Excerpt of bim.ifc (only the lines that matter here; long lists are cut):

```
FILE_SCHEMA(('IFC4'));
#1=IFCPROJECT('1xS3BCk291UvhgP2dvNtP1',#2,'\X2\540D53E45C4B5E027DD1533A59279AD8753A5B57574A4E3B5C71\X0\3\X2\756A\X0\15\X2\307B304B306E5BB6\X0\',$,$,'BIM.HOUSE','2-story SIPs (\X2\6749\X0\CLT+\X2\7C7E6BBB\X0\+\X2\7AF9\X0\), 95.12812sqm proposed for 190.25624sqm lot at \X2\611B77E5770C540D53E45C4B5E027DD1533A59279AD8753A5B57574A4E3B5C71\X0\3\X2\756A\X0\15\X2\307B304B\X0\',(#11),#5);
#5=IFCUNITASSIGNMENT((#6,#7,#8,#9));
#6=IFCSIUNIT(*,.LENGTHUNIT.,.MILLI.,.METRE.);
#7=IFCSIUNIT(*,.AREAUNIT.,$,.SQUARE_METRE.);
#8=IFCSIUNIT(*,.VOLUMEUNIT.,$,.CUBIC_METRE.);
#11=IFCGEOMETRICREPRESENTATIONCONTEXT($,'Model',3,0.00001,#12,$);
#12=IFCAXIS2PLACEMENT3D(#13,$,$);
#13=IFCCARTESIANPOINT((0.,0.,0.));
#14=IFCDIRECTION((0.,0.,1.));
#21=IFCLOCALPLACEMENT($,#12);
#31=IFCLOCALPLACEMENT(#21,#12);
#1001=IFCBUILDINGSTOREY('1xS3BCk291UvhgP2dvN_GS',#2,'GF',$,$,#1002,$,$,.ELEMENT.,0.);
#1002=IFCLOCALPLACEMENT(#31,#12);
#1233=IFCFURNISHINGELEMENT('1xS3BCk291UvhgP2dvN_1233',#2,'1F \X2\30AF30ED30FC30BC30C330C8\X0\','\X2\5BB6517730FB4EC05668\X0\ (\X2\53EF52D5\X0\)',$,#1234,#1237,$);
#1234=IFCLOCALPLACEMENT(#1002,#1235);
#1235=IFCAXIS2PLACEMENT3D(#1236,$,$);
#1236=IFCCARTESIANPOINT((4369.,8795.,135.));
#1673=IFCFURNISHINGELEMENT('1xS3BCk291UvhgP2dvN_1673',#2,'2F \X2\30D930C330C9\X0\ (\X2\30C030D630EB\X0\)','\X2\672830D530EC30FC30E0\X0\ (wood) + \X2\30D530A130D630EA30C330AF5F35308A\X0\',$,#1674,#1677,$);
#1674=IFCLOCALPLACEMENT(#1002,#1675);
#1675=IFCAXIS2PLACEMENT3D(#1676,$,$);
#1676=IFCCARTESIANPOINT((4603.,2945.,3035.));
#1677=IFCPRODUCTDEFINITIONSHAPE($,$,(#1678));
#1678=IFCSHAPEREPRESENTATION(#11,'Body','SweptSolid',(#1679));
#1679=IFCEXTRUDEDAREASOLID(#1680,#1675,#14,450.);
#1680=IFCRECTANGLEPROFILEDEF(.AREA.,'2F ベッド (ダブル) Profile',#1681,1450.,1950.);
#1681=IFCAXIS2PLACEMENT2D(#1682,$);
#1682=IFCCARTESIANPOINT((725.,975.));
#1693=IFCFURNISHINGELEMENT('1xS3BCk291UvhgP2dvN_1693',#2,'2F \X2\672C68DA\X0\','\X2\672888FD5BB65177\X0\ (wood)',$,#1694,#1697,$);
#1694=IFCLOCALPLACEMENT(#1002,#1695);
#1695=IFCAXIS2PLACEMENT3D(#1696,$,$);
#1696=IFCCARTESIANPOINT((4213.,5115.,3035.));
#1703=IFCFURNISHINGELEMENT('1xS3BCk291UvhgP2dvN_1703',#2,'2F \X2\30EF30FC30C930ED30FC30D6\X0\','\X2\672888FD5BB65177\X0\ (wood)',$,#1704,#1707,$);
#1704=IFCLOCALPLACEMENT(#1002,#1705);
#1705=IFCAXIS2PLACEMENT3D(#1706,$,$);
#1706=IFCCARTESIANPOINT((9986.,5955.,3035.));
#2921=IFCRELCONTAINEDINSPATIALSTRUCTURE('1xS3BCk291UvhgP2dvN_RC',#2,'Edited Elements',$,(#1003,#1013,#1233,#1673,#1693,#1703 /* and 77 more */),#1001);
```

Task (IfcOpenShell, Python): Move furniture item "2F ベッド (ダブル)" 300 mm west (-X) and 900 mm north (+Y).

```python
import ifcopenshell
import ifcopenshell.api.geometry
import ifcopenshell.util.placement

model = ifcopenshell.open("bim.ifc")

item = model.by_guid("1xS3BCk291UvhgP2dvN_1673")
matrix = ifcopenshell.util.placement.get_local_placement(item.ObjectPlacement)
matrix[0, 3] -= 300.0
matrix[1, 3] += 900.0
ifcopenshell.api.geometry.edit_object_placement(model, product=item, matrix=matrix, is_si=False)

print(ifcopenshell.util.placement.get_local_placement(item.ObjectPlacement).round(3) + 0.0)

model.write("bim_rev.ifc")
```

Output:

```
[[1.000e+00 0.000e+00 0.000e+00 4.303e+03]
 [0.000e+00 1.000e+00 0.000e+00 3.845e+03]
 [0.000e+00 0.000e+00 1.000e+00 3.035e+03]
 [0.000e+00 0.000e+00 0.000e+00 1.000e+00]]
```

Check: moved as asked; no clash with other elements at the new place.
